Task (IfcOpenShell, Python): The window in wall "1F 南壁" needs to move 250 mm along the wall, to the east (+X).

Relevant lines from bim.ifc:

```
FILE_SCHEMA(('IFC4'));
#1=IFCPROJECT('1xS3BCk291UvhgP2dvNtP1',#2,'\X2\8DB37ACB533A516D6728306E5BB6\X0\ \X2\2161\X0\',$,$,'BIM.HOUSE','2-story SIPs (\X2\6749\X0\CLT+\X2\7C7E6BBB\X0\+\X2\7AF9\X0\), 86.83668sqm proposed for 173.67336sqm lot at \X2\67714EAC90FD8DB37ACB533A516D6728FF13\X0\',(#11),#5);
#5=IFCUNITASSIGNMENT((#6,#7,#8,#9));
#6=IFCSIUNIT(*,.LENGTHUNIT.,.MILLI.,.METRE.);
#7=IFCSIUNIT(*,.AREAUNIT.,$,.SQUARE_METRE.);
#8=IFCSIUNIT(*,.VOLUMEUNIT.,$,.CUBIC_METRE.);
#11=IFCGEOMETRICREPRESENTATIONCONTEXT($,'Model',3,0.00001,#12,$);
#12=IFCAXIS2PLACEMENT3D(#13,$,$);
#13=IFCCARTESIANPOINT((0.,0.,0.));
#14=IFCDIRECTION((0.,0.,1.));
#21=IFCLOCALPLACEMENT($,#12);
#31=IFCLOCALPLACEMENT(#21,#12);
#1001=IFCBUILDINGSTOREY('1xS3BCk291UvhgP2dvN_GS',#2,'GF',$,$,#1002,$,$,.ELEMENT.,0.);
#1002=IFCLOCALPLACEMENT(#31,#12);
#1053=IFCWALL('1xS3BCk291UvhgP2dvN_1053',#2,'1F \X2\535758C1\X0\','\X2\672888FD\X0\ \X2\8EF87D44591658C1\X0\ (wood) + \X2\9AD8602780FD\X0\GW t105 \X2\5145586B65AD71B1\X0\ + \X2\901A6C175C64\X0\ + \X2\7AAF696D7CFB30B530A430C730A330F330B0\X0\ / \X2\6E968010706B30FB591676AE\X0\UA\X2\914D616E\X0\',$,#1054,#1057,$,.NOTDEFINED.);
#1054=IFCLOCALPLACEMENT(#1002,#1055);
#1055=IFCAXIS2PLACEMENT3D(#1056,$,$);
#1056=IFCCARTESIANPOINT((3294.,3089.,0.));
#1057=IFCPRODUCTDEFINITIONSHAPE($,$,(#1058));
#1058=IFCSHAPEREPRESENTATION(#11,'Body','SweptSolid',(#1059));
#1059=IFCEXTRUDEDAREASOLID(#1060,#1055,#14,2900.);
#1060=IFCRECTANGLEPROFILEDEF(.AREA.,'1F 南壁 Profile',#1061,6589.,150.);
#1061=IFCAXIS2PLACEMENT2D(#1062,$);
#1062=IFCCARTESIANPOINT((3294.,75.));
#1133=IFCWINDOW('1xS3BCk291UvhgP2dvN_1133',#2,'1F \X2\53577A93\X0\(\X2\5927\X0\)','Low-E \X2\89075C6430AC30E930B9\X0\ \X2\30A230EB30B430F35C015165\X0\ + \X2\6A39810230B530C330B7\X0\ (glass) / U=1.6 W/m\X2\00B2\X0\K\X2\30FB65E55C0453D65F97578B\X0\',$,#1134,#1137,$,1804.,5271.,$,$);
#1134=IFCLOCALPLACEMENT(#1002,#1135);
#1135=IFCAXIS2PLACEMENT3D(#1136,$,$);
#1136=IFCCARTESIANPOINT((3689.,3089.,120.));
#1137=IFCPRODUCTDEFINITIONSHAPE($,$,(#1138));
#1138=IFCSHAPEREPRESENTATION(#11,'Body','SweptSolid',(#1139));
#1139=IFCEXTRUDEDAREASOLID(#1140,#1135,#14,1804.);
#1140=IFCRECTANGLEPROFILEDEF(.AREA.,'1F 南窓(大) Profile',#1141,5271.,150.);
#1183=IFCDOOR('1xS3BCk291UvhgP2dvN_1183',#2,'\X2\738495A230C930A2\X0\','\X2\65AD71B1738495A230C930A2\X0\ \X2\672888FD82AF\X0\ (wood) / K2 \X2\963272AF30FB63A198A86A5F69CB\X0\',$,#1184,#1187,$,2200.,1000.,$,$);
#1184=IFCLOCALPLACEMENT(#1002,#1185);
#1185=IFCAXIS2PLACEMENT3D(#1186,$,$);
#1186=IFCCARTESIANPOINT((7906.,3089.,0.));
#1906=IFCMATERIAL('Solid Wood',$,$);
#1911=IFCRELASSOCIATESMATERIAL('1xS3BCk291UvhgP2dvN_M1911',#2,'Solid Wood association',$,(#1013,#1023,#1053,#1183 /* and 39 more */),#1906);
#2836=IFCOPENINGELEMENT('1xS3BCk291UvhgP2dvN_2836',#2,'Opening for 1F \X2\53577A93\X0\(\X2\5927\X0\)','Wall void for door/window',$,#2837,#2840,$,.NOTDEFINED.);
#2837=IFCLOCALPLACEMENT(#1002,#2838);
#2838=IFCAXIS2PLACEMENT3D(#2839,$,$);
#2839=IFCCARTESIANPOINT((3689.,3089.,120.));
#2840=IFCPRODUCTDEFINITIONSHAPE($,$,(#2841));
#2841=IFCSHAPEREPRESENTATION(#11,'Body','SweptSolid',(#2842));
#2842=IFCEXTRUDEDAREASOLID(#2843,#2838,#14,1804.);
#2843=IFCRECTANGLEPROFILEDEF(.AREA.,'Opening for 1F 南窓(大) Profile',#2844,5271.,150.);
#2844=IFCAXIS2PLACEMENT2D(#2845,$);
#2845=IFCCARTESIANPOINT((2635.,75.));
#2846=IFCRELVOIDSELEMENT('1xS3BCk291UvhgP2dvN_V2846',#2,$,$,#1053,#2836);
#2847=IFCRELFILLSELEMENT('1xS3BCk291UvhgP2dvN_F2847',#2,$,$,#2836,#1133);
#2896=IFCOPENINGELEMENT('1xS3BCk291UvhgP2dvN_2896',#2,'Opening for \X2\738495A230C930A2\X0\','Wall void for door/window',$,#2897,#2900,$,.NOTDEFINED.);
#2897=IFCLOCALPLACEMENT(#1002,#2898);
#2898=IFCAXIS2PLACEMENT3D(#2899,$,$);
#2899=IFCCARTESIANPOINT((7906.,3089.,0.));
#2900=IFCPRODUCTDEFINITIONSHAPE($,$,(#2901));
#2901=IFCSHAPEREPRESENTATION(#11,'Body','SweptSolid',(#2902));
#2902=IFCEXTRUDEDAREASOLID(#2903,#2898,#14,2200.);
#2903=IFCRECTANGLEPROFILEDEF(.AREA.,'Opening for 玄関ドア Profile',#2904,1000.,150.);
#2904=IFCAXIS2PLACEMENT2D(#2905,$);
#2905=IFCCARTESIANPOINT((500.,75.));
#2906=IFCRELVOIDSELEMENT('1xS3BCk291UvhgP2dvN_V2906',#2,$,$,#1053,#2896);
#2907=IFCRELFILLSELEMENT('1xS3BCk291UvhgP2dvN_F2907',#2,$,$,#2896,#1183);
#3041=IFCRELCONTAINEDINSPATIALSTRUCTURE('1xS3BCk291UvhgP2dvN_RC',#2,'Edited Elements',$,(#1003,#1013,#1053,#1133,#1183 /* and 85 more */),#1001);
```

```python
import ifcopenshell
import ifcopenshell.api.geometry
import ifcopenshell.util.placement
import ifcopenshell.util.unit

model = ifcopenshell.open("bim.ifc")
unit_scale = ifcopenshell.util.unit.calculate_unit_scale(model)

window = model.by_guid("1xS3BCk291UvhgP2dvN_1133")
opening = window.FillsVoids[0].RelatingOpeningElement
wall = opening.VoidsElements[0].RelatingBuildingElement

wall_matrix = ifcopenshell.util.placement.get_local_placement(wall.ObjectPlacement)
shift = wall_matrix[:3, 0] * 0.25 / unit_scale
before = ifcopenshell.util.placement.get_local_placement(window.ObjectPlacement)[:3, 3].copy()

# The window is not placed relative to its opening, so move both.
for product in (opening, window):
    matrix = ifcopenshell.util.placement.get_local_placement(product.ObjectPlacement)
    matrix[:3, 3] += shift
    ifcopenshell.api.geometry.edit_object_placement(model, product=product, matrix=matrix, is_si=False)

after = ifcopenshell.util.placement.get_local_placement(window.ObjectPlacement)[:3, 3]
print("window moved by", (after - before).round(3) + 0.0)

model.write("bim-out.ifc")
```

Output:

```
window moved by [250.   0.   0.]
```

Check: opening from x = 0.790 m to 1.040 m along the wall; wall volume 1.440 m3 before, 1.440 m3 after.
